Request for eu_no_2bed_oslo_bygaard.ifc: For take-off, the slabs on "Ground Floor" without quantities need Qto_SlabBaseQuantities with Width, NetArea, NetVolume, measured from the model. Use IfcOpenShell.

First a look at what the model holds.

```python
import ifcopenshell
import ifcopenshell.util.element
import ifcopenshell.util.unit

model = ifcopenshell.open("eu_no_2bed_oslo_bygaard.ifc")
print(model.schema)
for unit_type in ("LENGTHUNIT", "AREAUNIT", "VOLUMEUNIT"):
    print(unit_type, ifcopenshell.util.unit.calculate_unit_scale(model, unit_type))
storey = next(s for s in model.by_type("IfcBuildingStorey") if s.Name == "Ground Floor")
slabs = [e for e in ifcopenshell.util.element.get_decomposition(storey) if e.is_a("IfcSlab")]
for e in sorted(slabs, key=lambda e: e.id()):
    print(e.id(), e.is_a(), e.Name, list(ifcopenshell.util.element.get_psets(e, qtos_only=True)), sep=" | ")
```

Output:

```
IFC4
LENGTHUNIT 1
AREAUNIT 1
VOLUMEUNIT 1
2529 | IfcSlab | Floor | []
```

```python
import ifcopenshell
import ifcopenshell.api.pset
import ifcopenshell.geom
import ifcopenshell.util.element
import ifcopenshell.util.shape
import ifcopenshell.util.unit

model = ifcopenshell.open("eu_no_2bed_oslo_bygaard.ifc")
unit_scale = ifcopenshell.util.unit.calculate_unit_scale(model)
area_scale = ifcopenshell.util.unit.calculate_unit_scale(model, "AREAUNIT")
volume_scale = ifcopenshell.util.unit.calculate_unit_scale(model, "VOLUMEUNIT")
settings = ifcopenshell.geom.settings()

storey = next(s for s in model.by_type("IfcBuildingStorey") if s.Name == "Ground Floor")
slabs = [e for e in ifcopenshell.util.element.get_decomposition(storey) if e.is_a("IfcSlab")]

for e in sorted(slabs, key=lambda e: e.id()):
    if ifcopenshell.util.element.get_psets(e, qtos_only=True, should_inherit=False):
        continue
    # Geometry comes back in metres, in the element's own axes.
    shape = ifcopenshell.geom.create_shape(settings, e)
    values = {
        "Width": ifcopenshell.util.shape.get_z(shape.geometry) / unit_scale,
        "NetArea": ifcopenshell.util.shape.get_footprint_area(shape.geometry) / area_scale,
        "NetVolume": ifcopenshell.util.shape.get_volume(shape.geometry) / volume_scale,
    }
    qto = ifcopenshell.api.pset.add_qto(model, product=e, name="Qto_SlabBaseQuantities")
    ifcopenshell.api.pset.edit_qto(model, qto=qto, properties=values)
    print(e.id(), {k: round(v, 3) for k, v in values.items()})

model.write("eu_no_2bed_oslo_bygaard-out.ifc")
```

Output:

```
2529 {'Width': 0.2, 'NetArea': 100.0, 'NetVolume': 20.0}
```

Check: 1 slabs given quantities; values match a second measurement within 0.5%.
